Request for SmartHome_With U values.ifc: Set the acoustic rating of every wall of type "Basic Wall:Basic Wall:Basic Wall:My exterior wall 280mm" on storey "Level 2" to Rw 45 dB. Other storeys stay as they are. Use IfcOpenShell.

First a look at what the model holds.

```python
import ifcopenshell
import ifcopenshell.util.element

model = ifcopenshell.open("SmartHome_With U values.ifc")
print(model.schema)
storey = next(s for s in model.by_type("IfcBuildingStorey") if s.Name == "Level 2")
walls = [e for e in ifcopenshell.util.element.get_decomposition(storey) if e.is_a("IfcWall")]
seen = {}
for e in walls:
    element_type = ifcopenshell.util.element.get_type(e)
    key = (element_type.Name if element_type != e and element_type else None, ifcopenshell.util.element.get_pset(e, "Pset_WallCommon", "AcousticRating"))
    seen[key] = seen.get(key, 0) + 1
for (name, value), count in sorted(seen.items(), key=str):
    print(count, "x", name, "|", value)
```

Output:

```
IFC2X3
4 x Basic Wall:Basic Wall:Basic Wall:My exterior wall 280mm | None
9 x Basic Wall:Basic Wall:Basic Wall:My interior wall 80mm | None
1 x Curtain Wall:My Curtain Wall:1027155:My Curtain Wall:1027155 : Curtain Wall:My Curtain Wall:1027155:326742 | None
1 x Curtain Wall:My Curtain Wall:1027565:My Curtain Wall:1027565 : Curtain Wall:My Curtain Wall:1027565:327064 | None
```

```python
import ifcopenshell
import ifcopenshell.api.pset
import ifcopenshell.util.element

model = ifcopenshell.open("SmartHome_With U values.ifc")

storey = next(s for s in model.by_type("IfcBuildingStorey") if s.Name == "Level 2")
walls = [e for e in ifcopenshell.util.element.get_decomposition(storey) if e.is_a("IfcWall")]

count = 0
for e in walls:
    element_type = ifcopenshell.util.element.get_type(e)
    if element_type in (None, e) or element_type.Name != "Basic Wall:Basic Wall:Basic Wall:My exterior wall 280mm":
        continue
    # add_pset returns the element's existing set when there is one.
    pset = ifcopenshell.api.pset.add_pset(model, product=e, name="Pset_WallCommon")
    ifcopenshell.api.pset.edit_pset(model, pset=pset, properties={"AcousticRating": "Rw 45 dB"})
    count += 1

print(count, "walls updated")

model.write("SmartHome_With U values_edited.ifc")
```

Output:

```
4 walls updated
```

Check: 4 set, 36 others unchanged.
